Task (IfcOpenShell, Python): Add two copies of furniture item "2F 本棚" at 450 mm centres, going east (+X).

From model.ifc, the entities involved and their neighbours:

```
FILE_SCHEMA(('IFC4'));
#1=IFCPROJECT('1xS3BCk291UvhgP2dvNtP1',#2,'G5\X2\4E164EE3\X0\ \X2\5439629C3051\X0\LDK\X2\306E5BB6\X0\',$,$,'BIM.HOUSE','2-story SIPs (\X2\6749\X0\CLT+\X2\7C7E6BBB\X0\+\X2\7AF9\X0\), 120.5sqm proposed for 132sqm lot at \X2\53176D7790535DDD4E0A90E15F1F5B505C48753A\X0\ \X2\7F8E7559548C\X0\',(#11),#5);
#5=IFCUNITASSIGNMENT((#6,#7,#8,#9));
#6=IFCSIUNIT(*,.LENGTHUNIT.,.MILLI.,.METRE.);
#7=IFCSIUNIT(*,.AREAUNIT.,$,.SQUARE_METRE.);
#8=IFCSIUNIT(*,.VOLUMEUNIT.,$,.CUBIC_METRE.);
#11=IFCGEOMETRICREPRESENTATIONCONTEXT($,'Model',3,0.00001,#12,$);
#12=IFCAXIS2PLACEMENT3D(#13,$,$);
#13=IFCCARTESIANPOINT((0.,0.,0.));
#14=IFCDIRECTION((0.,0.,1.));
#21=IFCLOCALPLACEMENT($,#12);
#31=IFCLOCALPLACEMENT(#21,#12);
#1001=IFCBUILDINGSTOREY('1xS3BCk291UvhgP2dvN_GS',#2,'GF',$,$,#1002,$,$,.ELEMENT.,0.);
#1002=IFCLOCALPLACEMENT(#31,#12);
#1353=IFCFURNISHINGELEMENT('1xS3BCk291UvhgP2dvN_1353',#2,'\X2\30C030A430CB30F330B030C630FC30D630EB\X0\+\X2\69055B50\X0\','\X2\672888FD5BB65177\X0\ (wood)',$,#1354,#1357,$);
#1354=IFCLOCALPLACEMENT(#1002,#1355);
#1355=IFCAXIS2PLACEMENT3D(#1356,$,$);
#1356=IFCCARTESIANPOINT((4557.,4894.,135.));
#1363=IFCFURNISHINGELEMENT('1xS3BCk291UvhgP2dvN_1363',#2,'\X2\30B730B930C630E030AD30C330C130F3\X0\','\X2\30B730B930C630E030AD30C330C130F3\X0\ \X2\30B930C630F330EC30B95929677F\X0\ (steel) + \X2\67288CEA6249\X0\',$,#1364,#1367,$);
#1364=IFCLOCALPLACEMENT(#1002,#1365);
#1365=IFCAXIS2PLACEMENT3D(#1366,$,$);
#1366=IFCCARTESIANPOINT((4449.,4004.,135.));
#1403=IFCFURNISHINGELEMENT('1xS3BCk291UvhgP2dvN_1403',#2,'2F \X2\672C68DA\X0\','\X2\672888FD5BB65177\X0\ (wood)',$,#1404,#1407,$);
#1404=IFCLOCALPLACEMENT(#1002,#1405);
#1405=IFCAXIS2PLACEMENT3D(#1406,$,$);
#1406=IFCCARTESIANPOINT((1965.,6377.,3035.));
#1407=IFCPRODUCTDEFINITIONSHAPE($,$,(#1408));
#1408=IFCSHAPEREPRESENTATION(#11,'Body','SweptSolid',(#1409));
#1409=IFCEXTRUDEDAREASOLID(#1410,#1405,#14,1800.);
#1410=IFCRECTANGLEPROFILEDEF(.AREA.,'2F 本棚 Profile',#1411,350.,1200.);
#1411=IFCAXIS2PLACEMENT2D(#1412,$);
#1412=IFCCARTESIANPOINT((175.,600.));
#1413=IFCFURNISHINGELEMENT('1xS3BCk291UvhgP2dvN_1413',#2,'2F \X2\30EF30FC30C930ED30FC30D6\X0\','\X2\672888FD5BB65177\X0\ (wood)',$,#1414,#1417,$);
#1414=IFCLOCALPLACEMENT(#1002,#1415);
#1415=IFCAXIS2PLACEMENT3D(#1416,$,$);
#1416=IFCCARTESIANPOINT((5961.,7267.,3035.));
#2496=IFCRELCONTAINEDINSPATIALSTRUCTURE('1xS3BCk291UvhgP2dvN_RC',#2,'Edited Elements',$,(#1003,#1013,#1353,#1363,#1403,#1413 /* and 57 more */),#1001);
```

```python
import numpy as np
import ifcopenshell
import ifcopenshell.api.geometry
import ifcopenshell.api.root
import ifcopenshell.util.element
import ifcopenshell.util.placement
import ifcopenshell.util.unit

model = ifcopenshell.open("model.ifc")
unit_scale = ifcopenshell.util.unit.calculate_unit_scale(model)


def reuse_history(source, copy):
    """copy_class also copies each property set's owner history, people and application; keep the originals."""
    for rel in copy.IsDefinedBy:
        if rel.is_a("IfcRelDefinesByProperties") and (history := rel.RelatingPropertyDefinition.OwnerHistory):
            rel.RelatingPropertyDefinition.OwnerHistory = source.OwnerHistory
            ifcopenshell.util.element.remove_deep2(model, history)


source = model.by_guid("1xS3BCk291UvhgP2dvN_1403")
base = ifcopenshell.util.placement.get_local_placement(source.ObjectPlacement)
step = np.array([1.0, 0.0, 0.0]) * 0.45 / unit_scale

for i in range(1, 3):
    copy = ifcopenshell.api.root.copy_class(model, product=source)
    copy.Representation = ifcopenshell.util.element.copy_deep(
        model, source.Representation, exclude=["IfcGeometricRepresentationContext", "IfcRepresentationMap"]
    )
    reuse_history(source, copy)
    matrix = base.copy()
    matrix[:3, 3] += i * step
    print("added at", matrix[:3, 3].round(3) + 0.0)
    ifcopenshell.api.geometry.edit_object_placement(model, product=copy, matrix=matrix, is_si=False)

model.write("model_updated.ifc")
```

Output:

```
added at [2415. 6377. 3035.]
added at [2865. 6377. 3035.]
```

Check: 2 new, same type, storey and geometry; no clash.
